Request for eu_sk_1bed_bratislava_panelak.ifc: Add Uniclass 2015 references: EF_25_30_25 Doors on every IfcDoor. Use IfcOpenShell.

First a look at what the model holds.

```python
import ifcopenshell

model = ifcopenshell.open("eu_sk_1bed_bratislava_panelak.ifc")
print(model.schema)
print("classifications:", [c.Name for c in model.by_type("IfcClassification")])
for ifc_class in ("IfcDoor", "IfcRoof", "IfcStair", "IfcWall", "IfcWindow"):
    print(ifc_class, len(model.by_type(ifc_class)))
```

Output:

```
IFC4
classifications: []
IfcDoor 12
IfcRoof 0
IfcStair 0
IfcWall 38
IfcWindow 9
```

```python
import ifcopenshell
import ifcopenshell.api.classification

model = ifcopenshell.open("eu_sk_1bed_bratislava_panelak.ifc")

system = ifcopenshell.api.classification.add_classification(model, classification="Uniclass 2015")

codes = {
    "IfcDoor": ("EF_25_30_25", "Doors"),
}
for ifc_class, (code, name) in codes.items():
    products = model.by_type(ifc_class)
    ifcopenshell.api.classification.add_reference(
        model, products=products, classification=system, identification=code, name=name
    )
    print(code, len(products))

model.write("eu_sk_1bed_bratislava_panelak_v2.ifc")
```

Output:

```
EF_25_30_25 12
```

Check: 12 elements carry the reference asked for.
